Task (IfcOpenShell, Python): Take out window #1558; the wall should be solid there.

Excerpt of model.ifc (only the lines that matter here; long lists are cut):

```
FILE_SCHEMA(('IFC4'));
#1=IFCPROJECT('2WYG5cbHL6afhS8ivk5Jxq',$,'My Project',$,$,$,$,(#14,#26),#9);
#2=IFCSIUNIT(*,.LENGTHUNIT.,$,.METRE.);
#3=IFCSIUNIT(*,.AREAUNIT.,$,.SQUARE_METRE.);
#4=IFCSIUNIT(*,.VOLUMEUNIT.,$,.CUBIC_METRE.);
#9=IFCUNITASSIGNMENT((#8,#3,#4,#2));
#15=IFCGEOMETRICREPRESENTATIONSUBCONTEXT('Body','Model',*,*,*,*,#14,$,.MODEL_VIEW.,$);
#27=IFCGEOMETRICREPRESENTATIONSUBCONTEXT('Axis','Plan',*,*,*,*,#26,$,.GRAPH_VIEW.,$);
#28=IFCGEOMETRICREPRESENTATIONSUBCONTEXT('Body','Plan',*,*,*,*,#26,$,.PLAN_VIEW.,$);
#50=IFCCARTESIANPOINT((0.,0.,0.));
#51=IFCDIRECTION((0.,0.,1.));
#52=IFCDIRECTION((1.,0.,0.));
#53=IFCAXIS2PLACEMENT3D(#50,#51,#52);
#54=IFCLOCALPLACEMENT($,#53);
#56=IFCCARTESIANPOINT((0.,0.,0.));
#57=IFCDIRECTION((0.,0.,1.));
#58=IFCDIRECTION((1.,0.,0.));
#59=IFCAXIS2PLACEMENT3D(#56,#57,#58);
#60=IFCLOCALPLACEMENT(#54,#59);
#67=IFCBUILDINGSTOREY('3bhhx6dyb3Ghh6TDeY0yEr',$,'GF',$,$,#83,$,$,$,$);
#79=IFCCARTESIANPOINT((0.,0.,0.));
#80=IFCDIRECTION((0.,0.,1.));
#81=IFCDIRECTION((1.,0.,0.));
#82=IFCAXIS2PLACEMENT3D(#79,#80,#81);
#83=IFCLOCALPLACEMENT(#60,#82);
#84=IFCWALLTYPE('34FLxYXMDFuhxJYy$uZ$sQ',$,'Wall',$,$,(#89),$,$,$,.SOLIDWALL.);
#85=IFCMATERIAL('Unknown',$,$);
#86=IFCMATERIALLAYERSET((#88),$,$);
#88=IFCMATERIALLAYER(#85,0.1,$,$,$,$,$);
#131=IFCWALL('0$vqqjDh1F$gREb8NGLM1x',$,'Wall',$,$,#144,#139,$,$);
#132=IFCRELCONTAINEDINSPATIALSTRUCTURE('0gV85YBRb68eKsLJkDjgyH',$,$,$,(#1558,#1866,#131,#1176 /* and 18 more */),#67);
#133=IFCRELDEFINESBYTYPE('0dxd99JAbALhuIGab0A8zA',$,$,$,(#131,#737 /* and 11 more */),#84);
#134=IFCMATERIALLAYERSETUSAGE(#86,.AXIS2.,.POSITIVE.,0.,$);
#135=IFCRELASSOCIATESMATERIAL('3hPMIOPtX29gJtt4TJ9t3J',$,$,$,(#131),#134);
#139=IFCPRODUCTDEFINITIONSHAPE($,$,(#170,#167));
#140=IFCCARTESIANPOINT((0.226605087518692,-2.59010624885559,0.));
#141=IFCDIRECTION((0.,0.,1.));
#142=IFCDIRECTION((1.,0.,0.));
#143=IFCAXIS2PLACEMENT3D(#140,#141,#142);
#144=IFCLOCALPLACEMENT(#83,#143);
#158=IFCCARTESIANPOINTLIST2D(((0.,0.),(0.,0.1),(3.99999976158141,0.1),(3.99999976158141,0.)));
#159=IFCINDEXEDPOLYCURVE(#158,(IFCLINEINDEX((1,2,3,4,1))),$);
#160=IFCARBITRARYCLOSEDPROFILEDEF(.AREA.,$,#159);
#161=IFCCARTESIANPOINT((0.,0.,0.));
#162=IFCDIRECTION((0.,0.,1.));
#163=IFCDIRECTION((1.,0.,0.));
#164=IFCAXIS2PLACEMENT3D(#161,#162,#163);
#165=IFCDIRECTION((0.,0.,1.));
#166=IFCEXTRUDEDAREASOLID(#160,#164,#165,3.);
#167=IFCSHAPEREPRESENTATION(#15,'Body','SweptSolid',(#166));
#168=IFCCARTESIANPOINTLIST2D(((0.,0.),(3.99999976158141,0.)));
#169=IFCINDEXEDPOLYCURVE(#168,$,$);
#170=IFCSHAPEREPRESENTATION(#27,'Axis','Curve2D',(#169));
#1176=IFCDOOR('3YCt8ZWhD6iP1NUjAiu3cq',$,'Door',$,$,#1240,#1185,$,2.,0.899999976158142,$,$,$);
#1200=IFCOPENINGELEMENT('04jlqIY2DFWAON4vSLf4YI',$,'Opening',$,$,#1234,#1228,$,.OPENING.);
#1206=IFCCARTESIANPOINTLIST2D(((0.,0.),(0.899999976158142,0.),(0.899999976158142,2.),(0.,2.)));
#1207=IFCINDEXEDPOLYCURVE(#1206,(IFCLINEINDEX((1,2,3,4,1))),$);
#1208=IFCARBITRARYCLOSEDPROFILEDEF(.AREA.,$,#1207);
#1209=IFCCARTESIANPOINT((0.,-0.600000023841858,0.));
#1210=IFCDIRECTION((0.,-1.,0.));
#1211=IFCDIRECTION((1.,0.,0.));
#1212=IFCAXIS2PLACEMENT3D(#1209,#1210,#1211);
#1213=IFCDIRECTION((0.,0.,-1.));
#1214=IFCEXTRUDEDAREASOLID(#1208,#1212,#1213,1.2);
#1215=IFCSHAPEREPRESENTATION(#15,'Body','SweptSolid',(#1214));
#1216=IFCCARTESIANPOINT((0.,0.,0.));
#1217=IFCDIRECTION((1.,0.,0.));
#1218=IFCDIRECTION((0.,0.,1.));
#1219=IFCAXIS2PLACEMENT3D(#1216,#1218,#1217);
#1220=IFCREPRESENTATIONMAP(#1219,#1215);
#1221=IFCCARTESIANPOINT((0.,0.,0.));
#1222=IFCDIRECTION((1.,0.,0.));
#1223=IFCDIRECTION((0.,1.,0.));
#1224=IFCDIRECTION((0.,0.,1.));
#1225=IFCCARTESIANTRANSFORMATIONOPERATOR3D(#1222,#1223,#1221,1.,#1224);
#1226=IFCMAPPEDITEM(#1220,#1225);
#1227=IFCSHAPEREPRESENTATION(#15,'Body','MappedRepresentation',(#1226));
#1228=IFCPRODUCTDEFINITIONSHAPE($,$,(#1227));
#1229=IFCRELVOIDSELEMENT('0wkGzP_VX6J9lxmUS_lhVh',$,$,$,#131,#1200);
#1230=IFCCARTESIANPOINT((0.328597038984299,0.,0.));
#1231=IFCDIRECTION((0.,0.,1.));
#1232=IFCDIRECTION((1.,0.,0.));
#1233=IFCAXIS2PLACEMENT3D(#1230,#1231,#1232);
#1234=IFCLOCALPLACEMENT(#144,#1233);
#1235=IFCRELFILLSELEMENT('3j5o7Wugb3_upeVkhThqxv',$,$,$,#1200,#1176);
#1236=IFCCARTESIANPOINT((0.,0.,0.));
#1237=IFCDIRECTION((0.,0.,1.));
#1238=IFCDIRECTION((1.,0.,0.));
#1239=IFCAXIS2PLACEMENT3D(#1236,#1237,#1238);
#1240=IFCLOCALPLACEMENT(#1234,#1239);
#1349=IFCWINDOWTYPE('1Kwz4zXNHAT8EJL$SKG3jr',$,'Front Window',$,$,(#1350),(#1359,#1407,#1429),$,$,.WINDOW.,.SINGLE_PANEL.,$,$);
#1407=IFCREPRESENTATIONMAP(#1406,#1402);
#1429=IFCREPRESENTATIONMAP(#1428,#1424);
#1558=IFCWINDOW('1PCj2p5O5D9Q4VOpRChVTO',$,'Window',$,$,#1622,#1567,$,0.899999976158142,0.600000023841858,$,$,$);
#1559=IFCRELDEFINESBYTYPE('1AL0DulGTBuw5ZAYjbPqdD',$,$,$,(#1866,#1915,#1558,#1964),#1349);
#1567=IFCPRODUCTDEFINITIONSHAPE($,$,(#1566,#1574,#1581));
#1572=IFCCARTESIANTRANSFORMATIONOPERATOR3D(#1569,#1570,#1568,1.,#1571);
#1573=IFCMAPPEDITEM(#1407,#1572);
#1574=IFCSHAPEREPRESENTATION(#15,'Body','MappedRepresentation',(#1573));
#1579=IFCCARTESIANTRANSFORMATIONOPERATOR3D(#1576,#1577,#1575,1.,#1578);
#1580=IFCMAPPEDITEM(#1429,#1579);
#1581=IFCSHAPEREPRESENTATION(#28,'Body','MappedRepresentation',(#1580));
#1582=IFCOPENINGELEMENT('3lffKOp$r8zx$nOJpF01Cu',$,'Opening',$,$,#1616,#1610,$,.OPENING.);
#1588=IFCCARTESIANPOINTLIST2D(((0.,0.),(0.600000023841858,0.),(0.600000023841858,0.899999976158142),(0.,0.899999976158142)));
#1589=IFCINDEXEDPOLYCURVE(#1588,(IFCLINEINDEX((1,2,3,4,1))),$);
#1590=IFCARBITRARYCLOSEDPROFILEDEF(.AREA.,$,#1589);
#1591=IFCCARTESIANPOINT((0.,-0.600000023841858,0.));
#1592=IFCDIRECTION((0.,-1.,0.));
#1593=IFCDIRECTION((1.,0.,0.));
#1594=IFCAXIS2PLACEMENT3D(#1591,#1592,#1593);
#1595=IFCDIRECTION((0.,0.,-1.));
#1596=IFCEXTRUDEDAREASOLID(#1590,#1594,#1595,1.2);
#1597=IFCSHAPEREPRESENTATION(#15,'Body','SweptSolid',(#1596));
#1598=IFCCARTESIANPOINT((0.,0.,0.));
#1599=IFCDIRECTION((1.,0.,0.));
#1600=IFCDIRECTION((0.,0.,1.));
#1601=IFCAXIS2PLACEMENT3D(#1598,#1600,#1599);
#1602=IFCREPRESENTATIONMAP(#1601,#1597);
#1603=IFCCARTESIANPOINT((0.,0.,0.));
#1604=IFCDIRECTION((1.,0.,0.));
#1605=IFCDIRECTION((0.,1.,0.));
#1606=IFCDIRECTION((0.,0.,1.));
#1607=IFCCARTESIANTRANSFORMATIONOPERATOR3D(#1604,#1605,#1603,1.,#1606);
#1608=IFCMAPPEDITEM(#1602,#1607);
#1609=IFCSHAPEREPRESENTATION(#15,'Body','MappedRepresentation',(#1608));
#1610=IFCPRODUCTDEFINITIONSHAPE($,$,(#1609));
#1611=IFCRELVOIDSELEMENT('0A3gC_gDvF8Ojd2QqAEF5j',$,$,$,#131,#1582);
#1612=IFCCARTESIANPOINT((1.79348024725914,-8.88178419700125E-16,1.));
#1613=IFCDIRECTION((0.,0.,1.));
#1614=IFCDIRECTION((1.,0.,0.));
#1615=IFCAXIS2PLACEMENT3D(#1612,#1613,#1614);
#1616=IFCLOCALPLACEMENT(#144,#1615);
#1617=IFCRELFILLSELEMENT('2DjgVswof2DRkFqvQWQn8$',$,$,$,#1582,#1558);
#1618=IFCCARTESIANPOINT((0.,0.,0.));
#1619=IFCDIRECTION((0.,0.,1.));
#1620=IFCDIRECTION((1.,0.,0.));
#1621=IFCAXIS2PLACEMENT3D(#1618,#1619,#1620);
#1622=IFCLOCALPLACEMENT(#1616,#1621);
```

```python
import ifcopenshell
import ifcopenshell.api.feature
import ifcopenshell.api.root
import ifcopenshell.geom
import ifcopenshell.util.shape

model = ifcopenshell.open("model.ifc")
settings = ifcopenshell.geom.settings()


def volume(element):
    """Net volume in cubic metres, openings subtracted."""
    shape = ifcopenshell.geom.create_shape(settings, element)
    return ifcopenshell.util.shape.get_volume(shape.geometry)


window = model.by_id(1558)
opening = window.FillsVoids[0].RelatingOpeningElement
wall = opening.VoidsElements[0].RelatingBuildingElement
before = volume(wall)

ifcopenshell.api.root.remove_product(model, product=window)
ifcopenshell.api.feature.remove_feature(model, feature=opening)

after = volume(wall)

print(f"wall volume {before:.3f} -> {after:.3f} m3")

model.write("model_updated.ifc")
```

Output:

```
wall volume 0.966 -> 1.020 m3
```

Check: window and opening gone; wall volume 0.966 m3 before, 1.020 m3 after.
